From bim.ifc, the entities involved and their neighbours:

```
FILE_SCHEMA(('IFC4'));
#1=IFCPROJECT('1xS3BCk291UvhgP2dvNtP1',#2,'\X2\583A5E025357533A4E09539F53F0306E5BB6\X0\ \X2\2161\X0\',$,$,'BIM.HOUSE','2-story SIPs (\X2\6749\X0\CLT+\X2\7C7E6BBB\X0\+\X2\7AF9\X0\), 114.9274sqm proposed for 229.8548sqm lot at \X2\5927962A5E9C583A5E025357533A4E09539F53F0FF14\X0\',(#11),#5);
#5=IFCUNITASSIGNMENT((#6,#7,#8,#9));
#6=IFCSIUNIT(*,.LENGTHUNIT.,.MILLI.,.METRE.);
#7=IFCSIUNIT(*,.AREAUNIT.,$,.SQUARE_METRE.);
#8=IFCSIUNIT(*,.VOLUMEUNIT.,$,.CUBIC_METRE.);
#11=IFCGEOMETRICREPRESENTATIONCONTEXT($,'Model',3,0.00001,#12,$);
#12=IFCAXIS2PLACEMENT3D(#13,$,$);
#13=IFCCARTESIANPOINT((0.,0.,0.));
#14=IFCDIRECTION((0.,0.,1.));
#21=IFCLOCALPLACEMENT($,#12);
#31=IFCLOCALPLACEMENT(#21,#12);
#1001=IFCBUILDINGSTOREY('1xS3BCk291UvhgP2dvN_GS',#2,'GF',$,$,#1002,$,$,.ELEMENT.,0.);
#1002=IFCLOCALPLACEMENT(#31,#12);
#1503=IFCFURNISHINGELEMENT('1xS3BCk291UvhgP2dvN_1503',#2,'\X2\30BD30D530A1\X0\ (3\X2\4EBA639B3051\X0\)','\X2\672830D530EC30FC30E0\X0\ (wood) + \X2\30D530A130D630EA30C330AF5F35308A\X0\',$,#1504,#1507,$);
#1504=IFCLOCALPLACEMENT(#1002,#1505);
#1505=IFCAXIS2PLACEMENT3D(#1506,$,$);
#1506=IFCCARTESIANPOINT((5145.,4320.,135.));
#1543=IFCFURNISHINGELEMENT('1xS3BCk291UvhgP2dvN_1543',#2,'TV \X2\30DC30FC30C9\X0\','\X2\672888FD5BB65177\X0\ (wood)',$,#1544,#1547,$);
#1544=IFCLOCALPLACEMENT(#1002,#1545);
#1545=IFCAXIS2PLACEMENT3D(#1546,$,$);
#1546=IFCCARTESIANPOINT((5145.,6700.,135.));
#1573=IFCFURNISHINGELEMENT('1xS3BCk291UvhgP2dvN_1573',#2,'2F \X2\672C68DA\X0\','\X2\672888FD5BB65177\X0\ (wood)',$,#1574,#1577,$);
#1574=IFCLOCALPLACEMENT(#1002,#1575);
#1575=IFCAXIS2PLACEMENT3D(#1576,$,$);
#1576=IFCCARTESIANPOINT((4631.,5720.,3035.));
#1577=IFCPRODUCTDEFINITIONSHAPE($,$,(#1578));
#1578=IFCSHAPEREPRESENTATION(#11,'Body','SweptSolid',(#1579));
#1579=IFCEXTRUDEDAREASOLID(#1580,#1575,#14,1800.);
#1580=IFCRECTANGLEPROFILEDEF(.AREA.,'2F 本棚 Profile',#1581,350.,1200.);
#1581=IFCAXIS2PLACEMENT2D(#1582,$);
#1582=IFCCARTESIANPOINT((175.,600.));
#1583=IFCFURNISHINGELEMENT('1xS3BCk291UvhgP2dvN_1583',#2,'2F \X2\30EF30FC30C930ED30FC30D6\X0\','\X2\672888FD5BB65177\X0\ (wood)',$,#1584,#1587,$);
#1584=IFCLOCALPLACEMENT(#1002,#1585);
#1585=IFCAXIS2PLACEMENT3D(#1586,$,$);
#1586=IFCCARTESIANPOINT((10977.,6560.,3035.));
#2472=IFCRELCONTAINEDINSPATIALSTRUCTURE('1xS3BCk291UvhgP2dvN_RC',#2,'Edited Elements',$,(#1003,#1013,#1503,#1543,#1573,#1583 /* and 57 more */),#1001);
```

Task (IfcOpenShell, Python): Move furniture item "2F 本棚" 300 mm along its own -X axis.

```python
import ifcopenshell
import ifcopenshell.api.geometry
import ifcopenshell.util.placement
import ifcopenshell.util.unit

model = ifcopenshell.open("bim.ifc")
unit_scale = ifcopenshell.util.unit.calculate_unit_scale(model)

item = model.by_guid("1xS3BCk291UvhgP2dvN_1573")
matrix = ifcopenshell.util.placement.get_local_placement(item.ObjectPlacement)
matrix[:3, 3] -= matrix[:3, 0] * 0.3 / unit_scale
ifcopenshell.api.geometry.edit_object_placement(model, product=item, matrix=matrix, is_si=False)

print(ifcopenshell.util.placement.get_local_placement(item.ObjectPlacement).round(3) + 0.0)

model.write("bim_edited.ifc")
```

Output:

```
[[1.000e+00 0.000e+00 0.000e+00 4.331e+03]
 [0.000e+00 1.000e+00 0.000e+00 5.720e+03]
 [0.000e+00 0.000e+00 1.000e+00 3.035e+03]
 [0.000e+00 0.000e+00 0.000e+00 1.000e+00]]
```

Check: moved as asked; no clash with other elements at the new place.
